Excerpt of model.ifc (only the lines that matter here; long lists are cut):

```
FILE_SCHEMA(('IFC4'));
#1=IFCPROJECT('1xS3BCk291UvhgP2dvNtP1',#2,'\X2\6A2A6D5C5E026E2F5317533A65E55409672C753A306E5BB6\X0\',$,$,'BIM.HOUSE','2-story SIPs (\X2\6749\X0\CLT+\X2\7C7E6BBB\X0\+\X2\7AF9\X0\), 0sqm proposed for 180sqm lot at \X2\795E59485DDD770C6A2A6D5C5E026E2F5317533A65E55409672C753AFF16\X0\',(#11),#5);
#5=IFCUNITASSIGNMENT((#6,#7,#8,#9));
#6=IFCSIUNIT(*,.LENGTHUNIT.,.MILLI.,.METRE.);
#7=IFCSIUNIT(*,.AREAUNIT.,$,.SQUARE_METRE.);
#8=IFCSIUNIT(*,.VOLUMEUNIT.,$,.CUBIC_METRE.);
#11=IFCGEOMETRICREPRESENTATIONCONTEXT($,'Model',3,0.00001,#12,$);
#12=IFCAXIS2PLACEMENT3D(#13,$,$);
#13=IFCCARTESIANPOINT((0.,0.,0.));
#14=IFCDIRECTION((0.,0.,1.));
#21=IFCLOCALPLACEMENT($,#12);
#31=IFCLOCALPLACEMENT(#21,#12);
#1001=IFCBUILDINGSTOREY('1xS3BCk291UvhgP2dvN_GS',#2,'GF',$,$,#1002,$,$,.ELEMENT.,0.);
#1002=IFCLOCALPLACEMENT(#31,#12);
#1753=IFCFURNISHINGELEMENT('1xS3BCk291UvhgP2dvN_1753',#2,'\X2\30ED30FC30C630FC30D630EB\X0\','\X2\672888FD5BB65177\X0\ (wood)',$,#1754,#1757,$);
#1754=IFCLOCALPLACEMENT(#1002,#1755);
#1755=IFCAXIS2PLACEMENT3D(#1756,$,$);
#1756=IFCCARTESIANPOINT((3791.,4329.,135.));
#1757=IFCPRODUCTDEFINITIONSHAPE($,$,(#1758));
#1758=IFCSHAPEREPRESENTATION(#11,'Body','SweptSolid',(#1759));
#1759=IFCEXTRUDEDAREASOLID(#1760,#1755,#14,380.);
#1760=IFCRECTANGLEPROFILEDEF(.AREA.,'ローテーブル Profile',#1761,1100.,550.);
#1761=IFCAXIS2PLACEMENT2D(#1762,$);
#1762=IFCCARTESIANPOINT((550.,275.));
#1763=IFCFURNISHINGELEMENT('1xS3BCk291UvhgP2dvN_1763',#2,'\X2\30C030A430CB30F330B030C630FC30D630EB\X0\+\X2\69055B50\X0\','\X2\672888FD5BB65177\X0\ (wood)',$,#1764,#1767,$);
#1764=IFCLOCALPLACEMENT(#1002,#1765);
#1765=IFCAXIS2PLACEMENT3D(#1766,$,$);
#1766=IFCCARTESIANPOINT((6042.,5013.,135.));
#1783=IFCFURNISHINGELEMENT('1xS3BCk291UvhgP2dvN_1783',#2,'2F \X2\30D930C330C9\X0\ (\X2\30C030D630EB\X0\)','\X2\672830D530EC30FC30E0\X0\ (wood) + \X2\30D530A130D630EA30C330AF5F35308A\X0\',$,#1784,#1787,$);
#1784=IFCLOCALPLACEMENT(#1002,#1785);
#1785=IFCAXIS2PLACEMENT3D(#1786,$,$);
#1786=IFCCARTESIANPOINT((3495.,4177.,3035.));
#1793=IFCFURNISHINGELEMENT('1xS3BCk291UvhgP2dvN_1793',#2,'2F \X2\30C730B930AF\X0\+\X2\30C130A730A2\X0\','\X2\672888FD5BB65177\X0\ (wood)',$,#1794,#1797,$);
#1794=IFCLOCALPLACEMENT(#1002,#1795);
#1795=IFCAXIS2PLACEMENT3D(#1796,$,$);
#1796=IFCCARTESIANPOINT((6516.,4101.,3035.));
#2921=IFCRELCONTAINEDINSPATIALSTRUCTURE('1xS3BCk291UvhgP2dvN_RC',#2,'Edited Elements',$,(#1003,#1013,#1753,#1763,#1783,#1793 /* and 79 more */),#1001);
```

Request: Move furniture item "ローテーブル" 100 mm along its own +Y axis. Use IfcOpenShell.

```python
import ifcopenshell
import ifcopenshell.api.geometry
import ifcopenshell.util.placement
import ifcopenshell.util.unit

model = ifcopenshell.open("model.ifc")
unit_scale = ifcopenshell.util.unit.calculate_unit_scale(model)

item = model.by_guid("1xS3BCk291UvhgP2dvN_1753")
matrix = ifcopenshell.util.placement.get_local_placement(item.ObjectPlacement)
matrix[:3, 3] += matrix[:3, 1] * 0.1 / unit_scale
ifcopenshell.api.geometry.edit_object_placement(model, product=item, matrix=matrix, is_si=False)

print(ifcopenshell.util.placement.get_local_placement(item.ObjectPlacement).round(3) + 0.0)

model.write("model_v2.ifc")
```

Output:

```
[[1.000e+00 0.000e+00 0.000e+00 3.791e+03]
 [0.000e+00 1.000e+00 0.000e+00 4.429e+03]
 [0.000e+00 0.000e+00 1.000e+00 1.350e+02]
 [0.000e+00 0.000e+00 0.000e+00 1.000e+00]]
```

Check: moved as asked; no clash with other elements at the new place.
